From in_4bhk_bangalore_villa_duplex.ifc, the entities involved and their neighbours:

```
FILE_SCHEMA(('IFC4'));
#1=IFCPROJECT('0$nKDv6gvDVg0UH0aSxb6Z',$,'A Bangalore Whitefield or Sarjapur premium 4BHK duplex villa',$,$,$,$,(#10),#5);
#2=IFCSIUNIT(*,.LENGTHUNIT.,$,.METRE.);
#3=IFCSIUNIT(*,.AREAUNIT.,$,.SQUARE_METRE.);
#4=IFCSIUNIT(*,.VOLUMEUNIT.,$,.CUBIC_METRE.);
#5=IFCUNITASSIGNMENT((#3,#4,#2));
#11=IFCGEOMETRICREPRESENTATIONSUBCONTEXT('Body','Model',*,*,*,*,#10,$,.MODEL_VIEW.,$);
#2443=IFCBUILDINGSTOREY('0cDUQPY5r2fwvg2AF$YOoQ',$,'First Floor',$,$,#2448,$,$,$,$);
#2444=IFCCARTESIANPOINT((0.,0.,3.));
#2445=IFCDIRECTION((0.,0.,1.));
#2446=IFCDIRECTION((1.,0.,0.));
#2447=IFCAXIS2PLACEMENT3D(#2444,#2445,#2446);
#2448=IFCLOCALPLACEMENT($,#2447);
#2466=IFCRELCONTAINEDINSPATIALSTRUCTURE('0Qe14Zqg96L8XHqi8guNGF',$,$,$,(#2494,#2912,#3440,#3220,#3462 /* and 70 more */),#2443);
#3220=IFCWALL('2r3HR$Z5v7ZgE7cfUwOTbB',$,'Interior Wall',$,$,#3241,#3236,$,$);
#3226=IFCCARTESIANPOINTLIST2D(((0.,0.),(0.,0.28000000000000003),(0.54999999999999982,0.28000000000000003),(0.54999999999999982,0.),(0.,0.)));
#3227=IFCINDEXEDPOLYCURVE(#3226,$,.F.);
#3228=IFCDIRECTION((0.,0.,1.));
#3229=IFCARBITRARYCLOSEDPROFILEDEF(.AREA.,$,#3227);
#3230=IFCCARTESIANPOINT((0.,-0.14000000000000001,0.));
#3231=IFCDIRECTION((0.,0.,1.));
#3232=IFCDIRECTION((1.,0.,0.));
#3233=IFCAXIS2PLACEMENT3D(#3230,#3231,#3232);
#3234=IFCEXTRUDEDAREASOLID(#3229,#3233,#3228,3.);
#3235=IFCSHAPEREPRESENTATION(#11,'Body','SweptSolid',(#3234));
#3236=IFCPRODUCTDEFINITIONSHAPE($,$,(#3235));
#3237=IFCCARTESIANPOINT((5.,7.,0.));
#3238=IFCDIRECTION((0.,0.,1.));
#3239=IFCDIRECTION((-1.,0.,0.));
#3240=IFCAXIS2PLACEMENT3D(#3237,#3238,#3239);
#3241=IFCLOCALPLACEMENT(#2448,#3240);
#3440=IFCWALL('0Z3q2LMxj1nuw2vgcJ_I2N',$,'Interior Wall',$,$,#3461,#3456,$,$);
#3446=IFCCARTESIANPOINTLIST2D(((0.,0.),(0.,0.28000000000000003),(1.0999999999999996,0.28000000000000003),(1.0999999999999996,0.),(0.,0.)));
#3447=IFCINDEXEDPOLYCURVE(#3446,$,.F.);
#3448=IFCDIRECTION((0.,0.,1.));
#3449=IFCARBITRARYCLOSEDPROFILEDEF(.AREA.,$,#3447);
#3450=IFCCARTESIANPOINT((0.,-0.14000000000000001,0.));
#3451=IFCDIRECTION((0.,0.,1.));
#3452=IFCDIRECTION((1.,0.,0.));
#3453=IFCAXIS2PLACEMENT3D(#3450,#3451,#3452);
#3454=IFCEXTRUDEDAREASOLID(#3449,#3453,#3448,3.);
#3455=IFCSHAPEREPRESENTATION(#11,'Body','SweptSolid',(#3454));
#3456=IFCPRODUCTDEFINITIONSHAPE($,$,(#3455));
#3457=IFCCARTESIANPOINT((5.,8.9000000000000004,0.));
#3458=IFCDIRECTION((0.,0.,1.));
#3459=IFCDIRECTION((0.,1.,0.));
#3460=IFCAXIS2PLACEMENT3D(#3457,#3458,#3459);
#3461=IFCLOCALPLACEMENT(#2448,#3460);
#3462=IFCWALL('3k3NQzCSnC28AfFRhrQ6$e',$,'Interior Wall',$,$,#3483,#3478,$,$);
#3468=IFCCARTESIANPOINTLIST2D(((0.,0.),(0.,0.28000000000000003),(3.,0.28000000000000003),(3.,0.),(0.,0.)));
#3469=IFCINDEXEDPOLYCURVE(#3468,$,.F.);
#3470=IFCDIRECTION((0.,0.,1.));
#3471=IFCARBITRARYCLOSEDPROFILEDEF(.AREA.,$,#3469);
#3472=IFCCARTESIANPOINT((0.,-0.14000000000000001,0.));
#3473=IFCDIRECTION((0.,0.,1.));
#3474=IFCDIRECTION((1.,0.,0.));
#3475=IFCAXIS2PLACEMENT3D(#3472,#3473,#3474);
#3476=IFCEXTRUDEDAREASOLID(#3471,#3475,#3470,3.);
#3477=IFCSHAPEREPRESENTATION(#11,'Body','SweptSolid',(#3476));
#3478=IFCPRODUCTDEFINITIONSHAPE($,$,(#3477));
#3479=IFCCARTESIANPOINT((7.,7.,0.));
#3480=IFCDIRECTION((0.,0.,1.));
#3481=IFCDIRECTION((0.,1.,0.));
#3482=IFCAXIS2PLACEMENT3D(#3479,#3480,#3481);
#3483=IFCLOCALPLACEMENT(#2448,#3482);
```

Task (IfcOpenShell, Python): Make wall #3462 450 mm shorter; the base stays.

```python
import ifcopenshell
import ifcopenshell.geom
import ifcopenshell.util.representation
import ifcopenshell.util.shape
import ifcopenshell.util.unit

model = ifcopenshell.open("in_4bhk_bangalore_villa_duplex.ifc")
unit_scale = ifcopenshell.util.unit.calculate_unit_scale(model)
settings = ifcopenshell.geom.settings()


def volume(element):
    """Net volume in cubic metres, openings subtracted."""
    shape = ifcopenshell.geom.create_shape(settings, element)
    return ifcopenshell.util.shape.get_volume(shape.geometry)


wall = model.by_guid("3k3NQzCSnC28AfFRhrQ6$e")
before = volume(wall)

body = ifcopenshell.util.representation.get_representation(wall, "Model", "Body")
solid = body.Items[0]
old_height = solid.Depth
solid.Depth -= 0.45 / unit_scale
after = volume(wall)

print(f"height {old_height:g} -> {solid.Depth:g}, volume {before:.3f} -> {after:.3f} m3")

model.write("in_4bhk_bangalore_villa_duplex_updated.ifc")
```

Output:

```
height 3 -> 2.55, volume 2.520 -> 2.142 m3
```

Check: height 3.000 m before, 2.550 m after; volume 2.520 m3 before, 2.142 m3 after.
